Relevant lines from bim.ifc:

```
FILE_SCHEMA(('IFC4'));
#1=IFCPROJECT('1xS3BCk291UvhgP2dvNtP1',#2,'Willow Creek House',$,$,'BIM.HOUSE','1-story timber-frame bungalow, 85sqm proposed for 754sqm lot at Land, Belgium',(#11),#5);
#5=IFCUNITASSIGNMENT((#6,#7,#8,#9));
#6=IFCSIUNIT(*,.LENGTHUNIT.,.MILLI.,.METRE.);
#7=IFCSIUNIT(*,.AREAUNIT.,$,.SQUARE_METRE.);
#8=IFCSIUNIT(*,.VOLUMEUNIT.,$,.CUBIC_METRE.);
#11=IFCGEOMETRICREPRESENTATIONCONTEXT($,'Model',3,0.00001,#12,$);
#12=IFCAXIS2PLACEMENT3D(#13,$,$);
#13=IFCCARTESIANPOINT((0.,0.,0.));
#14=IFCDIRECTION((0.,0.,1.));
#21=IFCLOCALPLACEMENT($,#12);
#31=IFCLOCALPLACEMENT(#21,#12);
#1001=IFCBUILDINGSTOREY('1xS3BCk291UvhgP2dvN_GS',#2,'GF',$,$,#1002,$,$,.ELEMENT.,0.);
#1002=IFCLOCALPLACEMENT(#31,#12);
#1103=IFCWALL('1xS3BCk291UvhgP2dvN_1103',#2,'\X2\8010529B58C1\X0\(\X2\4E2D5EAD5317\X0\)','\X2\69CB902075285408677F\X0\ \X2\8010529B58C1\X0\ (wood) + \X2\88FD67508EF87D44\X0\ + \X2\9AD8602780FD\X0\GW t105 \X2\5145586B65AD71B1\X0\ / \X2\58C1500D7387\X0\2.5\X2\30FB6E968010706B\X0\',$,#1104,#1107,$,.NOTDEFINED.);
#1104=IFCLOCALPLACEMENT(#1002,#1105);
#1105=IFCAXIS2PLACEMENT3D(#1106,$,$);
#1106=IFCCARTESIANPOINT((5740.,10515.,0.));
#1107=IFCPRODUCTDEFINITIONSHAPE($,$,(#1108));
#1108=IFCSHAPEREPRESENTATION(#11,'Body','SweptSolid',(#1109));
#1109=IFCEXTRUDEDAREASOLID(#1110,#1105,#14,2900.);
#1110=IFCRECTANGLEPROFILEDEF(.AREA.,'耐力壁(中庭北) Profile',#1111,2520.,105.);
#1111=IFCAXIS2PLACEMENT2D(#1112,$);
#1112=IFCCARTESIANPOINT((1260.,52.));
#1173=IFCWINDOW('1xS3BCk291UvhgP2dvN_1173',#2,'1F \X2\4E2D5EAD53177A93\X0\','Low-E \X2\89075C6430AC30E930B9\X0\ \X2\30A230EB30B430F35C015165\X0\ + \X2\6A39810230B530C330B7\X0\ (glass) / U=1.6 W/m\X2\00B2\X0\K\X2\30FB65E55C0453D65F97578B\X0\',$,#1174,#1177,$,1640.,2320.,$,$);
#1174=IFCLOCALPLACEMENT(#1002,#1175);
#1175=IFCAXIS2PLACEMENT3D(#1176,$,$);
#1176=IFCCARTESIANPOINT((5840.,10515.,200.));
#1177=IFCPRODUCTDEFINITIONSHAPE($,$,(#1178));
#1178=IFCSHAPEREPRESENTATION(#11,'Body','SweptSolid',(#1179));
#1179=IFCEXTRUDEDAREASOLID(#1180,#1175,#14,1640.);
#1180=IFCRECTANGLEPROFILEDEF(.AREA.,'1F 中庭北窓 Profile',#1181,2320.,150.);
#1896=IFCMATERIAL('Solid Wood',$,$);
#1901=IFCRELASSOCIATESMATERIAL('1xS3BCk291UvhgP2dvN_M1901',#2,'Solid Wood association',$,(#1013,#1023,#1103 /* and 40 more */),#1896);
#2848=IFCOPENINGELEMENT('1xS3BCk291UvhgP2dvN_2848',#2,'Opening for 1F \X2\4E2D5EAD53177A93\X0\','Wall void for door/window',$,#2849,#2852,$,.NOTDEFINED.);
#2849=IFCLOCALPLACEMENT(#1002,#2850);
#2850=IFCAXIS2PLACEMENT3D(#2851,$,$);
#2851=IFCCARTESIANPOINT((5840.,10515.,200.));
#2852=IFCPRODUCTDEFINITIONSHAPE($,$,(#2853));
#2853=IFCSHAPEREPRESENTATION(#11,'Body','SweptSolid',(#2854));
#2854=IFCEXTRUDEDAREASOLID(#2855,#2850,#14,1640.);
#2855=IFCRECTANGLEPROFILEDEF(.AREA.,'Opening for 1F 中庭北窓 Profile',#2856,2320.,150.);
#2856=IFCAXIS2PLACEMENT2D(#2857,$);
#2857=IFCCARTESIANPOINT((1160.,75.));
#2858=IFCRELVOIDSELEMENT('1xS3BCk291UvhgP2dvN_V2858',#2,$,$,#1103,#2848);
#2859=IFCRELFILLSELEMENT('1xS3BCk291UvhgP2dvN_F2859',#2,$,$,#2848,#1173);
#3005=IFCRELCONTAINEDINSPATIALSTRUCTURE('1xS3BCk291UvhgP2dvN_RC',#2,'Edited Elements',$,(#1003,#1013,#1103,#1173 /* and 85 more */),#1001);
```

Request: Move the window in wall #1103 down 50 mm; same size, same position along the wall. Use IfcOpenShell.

```python
import numpy as np
import ifcopenshell
import ifcopenshell.api.geometry
import ifcopenshell.util.placement
import ifcopenshell.util.unit

model = ifcopenshell.open("bim.ifc")
unit_scale = ifcopenshell.util.unit.calculate_unit_scale(model)

window = model.by_guid("1xS3BCk291UvhgP2dvN_1173")
opening = window.FillsVoids[0].RelatingOpeningElement
dz = -50.0

shift = np.array([0.0, 0.0, dz])
# The window is not placed relative to its opening, so move both.
for product in (opening, window):
    matrix = ifcopenshell.util.placement.get_local_placement(product.ObjectPlacement)
    matrix[:3, 3] += shift
    ifcopenshell.api.geometry.edit_object_placement(model, product=product, matrix=matrix, is_si=False)

print(f"moved by {dz * unit_scale:+.3f} m")

model.write("bim_updated.ifc")
```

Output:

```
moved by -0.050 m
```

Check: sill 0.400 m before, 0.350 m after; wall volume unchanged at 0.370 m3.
